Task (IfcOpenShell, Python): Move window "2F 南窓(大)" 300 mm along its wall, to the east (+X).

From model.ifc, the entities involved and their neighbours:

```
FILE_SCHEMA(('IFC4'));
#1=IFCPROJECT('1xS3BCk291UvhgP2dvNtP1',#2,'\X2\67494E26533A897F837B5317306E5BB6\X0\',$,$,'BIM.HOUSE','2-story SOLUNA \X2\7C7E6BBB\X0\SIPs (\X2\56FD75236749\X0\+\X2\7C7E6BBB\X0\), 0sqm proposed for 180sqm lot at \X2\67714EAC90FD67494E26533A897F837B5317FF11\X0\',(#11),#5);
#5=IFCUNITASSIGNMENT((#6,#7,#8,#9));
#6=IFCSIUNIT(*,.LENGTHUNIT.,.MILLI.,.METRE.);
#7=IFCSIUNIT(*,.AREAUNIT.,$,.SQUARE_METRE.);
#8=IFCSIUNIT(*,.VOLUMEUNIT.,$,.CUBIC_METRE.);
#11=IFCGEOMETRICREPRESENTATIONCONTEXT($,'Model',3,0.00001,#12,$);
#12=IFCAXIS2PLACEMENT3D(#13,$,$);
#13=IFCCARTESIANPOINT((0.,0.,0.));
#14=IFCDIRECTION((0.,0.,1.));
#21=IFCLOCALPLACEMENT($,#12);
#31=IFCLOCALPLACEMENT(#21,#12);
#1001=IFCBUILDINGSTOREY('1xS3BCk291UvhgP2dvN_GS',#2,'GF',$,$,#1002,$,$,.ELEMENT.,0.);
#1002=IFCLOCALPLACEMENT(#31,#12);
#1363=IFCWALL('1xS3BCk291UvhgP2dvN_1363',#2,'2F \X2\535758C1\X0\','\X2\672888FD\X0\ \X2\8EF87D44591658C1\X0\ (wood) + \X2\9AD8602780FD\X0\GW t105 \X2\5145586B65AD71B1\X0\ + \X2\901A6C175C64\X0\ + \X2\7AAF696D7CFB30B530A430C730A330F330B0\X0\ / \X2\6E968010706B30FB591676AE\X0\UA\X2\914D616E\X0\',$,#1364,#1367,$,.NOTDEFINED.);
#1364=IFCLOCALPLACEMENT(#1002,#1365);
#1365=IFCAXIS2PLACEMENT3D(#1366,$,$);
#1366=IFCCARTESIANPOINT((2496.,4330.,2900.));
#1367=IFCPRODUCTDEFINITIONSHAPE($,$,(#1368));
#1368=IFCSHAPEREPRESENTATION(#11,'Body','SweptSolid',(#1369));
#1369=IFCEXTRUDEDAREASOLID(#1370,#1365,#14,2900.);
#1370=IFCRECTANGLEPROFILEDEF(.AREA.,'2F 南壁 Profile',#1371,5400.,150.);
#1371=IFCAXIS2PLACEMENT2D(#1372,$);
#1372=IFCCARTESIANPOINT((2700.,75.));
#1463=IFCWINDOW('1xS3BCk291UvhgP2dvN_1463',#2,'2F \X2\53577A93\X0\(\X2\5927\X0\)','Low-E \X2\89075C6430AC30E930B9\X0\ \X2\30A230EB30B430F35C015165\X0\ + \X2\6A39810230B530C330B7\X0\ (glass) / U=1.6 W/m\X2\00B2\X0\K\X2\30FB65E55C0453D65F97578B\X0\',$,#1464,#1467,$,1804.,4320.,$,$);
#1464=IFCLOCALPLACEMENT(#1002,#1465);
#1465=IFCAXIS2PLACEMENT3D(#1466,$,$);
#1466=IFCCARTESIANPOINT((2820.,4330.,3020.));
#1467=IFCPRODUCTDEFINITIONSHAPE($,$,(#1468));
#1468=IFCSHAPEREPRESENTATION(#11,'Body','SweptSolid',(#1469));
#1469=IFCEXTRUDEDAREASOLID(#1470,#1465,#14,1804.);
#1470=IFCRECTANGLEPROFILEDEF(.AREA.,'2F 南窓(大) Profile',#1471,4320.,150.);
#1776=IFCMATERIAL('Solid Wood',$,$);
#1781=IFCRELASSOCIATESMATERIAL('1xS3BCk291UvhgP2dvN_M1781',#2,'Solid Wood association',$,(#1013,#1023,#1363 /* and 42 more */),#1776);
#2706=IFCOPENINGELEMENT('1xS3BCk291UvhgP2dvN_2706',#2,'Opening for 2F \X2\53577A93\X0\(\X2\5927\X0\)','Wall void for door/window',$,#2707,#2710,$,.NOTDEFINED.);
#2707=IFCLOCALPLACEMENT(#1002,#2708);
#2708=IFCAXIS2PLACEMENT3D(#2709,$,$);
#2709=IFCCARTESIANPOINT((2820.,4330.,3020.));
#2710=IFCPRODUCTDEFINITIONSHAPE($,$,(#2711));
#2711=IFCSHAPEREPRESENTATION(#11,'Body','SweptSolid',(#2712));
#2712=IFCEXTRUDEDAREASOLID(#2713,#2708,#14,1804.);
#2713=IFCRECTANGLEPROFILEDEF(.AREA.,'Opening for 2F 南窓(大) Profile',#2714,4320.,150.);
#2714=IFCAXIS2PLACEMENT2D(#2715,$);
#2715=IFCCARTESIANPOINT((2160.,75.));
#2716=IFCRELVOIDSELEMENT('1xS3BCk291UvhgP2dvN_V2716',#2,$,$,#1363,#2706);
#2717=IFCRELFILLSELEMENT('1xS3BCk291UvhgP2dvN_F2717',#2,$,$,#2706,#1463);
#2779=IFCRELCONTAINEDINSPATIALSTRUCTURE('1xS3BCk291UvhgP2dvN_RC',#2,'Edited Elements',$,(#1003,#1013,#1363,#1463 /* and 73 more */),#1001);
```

```python
import ifcopenshell
import ifcopenshell.api.geometry
import ifcopenshell.util.placement
import ifcopenshell.util.unit

model = ifcopenshell.open("model.ifc")
unit_scale = ifcopenshell.util.unit.calculate_unit_scale(model)

window = model.by_guid("1xS3BCk291UvhgP2dvN_1463")
opening = window.FillsVoids[0].RelatingOpeningElement
wall = opening.VoidsElements[0].RelatingBuildingElement

wall_matrix = ifcopenshell.util.placement.get_local_placement(wall.ObjectPlacement)
shift = wall_matrix[:3, 0] * 0.3 / unit_scale
before = ifcopenshell.util.placement.get_local_placement(window.ObjectPlacement)[:3, 3].copy()

# The window is not placed relative to its opening, so move both.
for product in (opening, window):
    matrix = ifcopenshell.util.placement.get_local_placement(product.ObjectPlacement)
    matrix[:3, 3] += shift
    ifcopenshell.api.geometry.edit_object_placement(model, product=product, matrix=matrix, is_si=False)

after = ifcopenshell.util.placement.get_local_placement(window.ObjectPlacement)[:3, 3]
print("window moved by", (after - before).round(3) + 0.0)

model.write("model_rev.ifc")
```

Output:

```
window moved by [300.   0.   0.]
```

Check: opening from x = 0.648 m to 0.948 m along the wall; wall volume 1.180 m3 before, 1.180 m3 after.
